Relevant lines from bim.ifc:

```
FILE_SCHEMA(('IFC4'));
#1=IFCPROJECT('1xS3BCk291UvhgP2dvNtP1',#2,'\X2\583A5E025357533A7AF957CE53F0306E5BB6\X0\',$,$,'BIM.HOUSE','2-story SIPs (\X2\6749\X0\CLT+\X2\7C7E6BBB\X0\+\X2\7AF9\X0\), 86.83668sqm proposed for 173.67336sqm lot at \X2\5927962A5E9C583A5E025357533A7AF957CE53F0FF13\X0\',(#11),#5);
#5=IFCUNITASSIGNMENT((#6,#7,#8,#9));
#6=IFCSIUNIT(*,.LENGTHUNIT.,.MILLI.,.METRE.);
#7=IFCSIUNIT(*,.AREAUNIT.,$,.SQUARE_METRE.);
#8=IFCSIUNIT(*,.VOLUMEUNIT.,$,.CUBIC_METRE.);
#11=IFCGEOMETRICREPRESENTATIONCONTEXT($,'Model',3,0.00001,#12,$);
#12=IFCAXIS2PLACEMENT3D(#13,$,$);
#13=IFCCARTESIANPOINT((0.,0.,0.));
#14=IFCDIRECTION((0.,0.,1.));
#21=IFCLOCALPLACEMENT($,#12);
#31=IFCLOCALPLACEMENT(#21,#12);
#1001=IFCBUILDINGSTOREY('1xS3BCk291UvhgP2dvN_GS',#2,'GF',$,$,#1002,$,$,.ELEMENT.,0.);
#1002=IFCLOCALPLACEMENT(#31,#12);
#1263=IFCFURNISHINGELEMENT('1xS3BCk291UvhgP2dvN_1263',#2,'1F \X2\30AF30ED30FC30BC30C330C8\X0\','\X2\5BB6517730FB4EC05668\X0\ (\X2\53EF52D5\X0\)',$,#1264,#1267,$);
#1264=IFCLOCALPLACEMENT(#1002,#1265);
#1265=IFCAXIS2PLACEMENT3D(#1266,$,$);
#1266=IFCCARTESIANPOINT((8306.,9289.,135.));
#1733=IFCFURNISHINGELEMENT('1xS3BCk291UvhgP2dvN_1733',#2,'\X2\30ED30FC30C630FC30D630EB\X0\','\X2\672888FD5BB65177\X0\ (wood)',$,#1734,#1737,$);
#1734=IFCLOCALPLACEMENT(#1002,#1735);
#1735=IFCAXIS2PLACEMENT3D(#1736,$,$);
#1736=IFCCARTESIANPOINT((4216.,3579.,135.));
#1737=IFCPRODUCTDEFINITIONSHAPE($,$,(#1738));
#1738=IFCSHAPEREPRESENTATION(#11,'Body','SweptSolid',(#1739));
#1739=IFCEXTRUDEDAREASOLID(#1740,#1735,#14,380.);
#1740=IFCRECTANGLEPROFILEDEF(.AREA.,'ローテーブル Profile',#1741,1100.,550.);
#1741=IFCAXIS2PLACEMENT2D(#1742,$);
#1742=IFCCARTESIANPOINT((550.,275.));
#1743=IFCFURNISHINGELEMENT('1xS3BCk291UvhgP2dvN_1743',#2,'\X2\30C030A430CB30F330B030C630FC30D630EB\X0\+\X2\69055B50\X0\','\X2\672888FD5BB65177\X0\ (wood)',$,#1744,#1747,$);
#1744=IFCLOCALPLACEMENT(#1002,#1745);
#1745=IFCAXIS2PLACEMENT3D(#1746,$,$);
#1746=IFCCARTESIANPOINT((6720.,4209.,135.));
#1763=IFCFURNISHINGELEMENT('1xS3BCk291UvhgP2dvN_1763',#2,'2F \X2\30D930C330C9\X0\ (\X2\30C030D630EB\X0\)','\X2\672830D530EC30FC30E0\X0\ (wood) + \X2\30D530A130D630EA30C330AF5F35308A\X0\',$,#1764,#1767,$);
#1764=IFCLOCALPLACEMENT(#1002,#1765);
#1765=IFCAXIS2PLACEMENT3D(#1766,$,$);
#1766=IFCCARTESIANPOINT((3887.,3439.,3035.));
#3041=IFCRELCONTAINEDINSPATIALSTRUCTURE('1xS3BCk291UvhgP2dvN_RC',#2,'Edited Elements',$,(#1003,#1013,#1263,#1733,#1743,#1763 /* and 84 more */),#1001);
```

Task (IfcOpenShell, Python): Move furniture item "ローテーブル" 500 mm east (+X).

```python
import ifcopenshell
import ifcopenshell.api.geometry
import ifcopenshell.util.placement
import ifcopenshell.util.unit

model = ifcopenshell.open("bim.ifc")
unit_scale = ifcopenshell.util.unit.calculate_unit_scale(model)

item = model.by_id(1733)
matrix = ifcopenshell.util.placement.get_local_placement(item.ObjectPlacement)
matrix[0, 3] += 0.5 / unit_scale
ifcopenshell.api.geometry.edit_object_placement(model, product=item, matrix=matrix, is_si=False)

print(ifcopenshell.util.placement.get_local_placement(item.ObjectPlacement).round(3) + 0.0)

model.write("bim_v2.ifc")
```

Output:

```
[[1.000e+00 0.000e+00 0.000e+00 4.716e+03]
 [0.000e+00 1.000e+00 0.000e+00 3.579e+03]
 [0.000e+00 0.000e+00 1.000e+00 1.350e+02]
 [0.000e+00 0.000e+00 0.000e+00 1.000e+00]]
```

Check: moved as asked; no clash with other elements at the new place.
